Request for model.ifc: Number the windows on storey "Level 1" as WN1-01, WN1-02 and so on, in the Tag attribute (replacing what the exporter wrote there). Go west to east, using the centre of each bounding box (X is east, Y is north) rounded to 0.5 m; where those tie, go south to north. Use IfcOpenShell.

First a look at what the model holds.

```python
import ifcopenshell
import ifcopenshell.util.element
import ifcopenshell.util.placement

model = ifcopenshell.open("model.ifc")
print(model.schema)
storey = next(s for s in model.by_type("IfcBuildingStorey") if s.Name == "Level 1")
windows = [e for e in ifcopenshell.util.element.get_decomposition(storey) if e.is_a("IfcWindow")]
for e in sorted(windows, key=lambda e: e.id()):
    origin = ifcopenshell.util.placement.get_local_placement(e.ObjectPlacement)[:3, 3]
    print(e.id(), e.Tag, e.Name, origin.round(2) + 0.0, sep=" | ")
```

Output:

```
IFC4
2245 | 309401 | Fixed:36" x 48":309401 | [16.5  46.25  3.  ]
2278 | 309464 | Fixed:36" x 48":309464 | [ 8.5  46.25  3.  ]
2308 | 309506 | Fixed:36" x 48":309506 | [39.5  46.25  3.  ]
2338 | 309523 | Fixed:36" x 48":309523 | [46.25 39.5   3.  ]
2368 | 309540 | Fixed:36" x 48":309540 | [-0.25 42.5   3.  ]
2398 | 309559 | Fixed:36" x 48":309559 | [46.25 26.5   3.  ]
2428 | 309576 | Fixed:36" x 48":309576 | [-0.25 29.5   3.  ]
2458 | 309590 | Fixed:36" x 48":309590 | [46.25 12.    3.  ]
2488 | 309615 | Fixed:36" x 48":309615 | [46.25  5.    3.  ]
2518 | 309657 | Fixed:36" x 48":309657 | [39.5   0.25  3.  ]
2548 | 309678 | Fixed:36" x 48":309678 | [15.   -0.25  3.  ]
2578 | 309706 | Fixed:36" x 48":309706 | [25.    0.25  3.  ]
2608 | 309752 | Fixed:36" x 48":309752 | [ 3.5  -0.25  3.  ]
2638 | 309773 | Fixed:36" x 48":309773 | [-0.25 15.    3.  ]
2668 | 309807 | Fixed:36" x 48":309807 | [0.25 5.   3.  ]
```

```python
import ifcopenshell
import ifcopenshell.geom
import ifcopenshell.util.element
import ifcopenshell.util.shape

model = ifcopenshell.open("model.ifc")
settings = ifcopenshell.geom.settings()
settings.set("use-world-coords", True)


def centre(element):
    shape = ifcopenshell.geom.create_shape(settings, element)
    return ifcopenshell.util.shape.get_bbox_centroid(shape.geometry)


storey = next(s for s in model.by_type("IfcBuildingStorey") if s.Name == "Level 1")
windows = [e for e in ifcopenshell.util.element.get_decomposition(storey) if e.is_a("IfcWindow")]

# Insertion points can sit at a corner or the storey origin, so sort by the geometry (in metres).
centres = {e: centre(e) for e in windows}
windows.sort(key=lambda e: (round(centres[e][0] / 0.5), centres[e][1]))

for i, e in enumerate(windows, start=1):
    number = f"WN1-{i:02d}"
    e.Tag = number
    print(e.id(), number)

model.write("model_rev.ifc")
```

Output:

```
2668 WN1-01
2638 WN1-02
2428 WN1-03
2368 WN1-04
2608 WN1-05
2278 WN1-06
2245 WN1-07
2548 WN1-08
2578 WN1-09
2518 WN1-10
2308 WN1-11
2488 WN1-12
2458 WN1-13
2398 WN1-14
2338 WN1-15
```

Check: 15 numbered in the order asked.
